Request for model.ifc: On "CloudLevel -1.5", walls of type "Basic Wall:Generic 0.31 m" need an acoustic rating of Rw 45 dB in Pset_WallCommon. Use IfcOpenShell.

First a look at what the model holds.

```python
import ifcopenshell
import ifcopenshell.util.element

model = ifcopenshell.open("model.ifc")
print(model.schema)
storey = next(s for s in model.by_type("IfcBuildingStorey") if s.Name == "CloudLevel -1.5")
walls = [e for e in ifcopenshell.util.element.get_decomposition(storey) if e.is_a("IfcWall")]
seen = {}
for e in walls:
    element_type = ifcopenshell.util.element.get_type(e)
    key = (element_type.Name if element_type != e and element_type else None, ifcopenshell.util.element.get_pset(e, "Pset_WallCommon", "AcousticRating"))
    seen[key] = seen.get(key, 0) + 1
for (name, value), count in sorted(seen.items(), key=str):
    print(count, "x", name, "|", value)
```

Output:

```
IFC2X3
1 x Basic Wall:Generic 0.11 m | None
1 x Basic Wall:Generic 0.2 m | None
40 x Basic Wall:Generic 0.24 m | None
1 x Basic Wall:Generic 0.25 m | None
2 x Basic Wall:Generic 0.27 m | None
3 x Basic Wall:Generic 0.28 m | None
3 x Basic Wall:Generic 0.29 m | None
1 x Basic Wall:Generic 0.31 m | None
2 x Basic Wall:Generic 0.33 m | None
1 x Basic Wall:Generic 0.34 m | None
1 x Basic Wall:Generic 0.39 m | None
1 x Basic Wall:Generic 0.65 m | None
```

```python
import ifcopenshell
import ifcopenshell.api.pset
import ifcopenshell.util.element

model = ifcopenshell.open("model.ifc")

storey = next(s for s in model.by_type("IfcBuildingStorey") if s.Name == "CloudLevel -1.5")
walls = [e for e in ifcopenshell.util.element.get_decomposition(storey) if e.is_a("IfcWall")]

count = 0
for e in walls:
    element_type = ifcopenshell.util.element.get_type(e)
    if element_type in (None, e) or element_type.Name != "Basic Wall:Generic 0.31 m":
        continue
    # add_pset returns the element's existing set when there is one.
    pset = ifcopenshell.api.pset.add_pset(model, product=e, name="Pset_WallCommon")
    ifcopenshell.api.pset.edit_pset(model, pset=pset, properties={"AcousticRating": "Rw 45 dB"})
    count += 1

print(count, "walls updated")

model.write("model_edited.ifc")
```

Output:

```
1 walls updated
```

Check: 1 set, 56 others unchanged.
